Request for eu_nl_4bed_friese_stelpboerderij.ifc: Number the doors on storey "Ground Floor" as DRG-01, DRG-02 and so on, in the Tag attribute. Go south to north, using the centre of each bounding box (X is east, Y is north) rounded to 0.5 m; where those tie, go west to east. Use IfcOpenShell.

First a look at what the model holds.

```python
import ifcopenshell
import ifcopenshell.util.element
import ifcopenshell.util.placement

model = ifcopenshell.open("eu_nl_4bed_friese_stelpboerderij.ifc")
print(model.schema)
storey = next(s for s in model.by_type("IfcBuildingStorey") if s.Name == "Ground Floor")
doors = [e for e in ifcopenshell.util.element.get_decomposition(storey) if e.is_a("IfcDoor")]
for e in sorted(doors, key=lambda e: e.id()):
    origin = ifcopenshell.util.placement.get_local_placement(e.ObjectPlacement)[:3, 3]
    print(e.id(), e.Tag, e.Name, origin.round(2) + 0.0, sep=" | ")
```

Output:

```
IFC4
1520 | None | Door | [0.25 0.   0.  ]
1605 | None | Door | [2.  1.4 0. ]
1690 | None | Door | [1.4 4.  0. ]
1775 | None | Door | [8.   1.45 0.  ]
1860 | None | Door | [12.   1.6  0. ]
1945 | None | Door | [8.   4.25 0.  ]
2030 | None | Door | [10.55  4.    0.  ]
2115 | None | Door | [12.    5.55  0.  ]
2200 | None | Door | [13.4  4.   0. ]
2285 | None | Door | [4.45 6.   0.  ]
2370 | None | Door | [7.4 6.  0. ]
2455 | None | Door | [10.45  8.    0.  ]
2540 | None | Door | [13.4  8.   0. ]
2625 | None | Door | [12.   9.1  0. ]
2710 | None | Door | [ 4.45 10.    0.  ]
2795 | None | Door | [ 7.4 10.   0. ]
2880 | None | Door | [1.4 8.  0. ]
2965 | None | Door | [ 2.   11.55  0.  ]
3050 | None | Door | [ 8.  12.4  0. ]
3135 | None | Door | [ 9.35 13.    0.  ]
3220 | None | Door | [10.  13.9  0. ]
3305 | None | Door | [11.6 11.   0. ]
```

```python
import ifcopenshell
import ifcopenshell.geom
import ifcopenshell.util.element
import ifcopenshell.util.shape

model = ifcopenshell.open("eu_nl_4bed_friese_stelpboerderij.ifc")
settings = ifcopenshell.geom.settings()
settings.set("use-world-coords", True)


def centre(element):
    shape = ifcopenshell.geom.create_shape(settings, element)
    return ifcopenshell.util.shape.get_bbox_centroid(shape.geometry)


storey = next(s for s in model.by_type("IfcBuildingStorey") if s.Name == "Ground Floor")
doors = [e for e in ifcopenshell.util.element.get_decomposition(storey) if e.is_a("IfcDoor")]

# Insertion points can sit at a corner or the storey origin, so sort by the geometry (in metres).
centres = {e: centre(e) for e in doors}
doors.sort(key=lambda e: (round(centres[e][1] / 0.5), centres[e][0]))

for i, e in enumerate(doors, start=1):
    number = f"DRG-{i:02d}"
    e.Tag = number
    print(e.id(), number)

model.write("eu_nl_4bed_friese_stelpboerderij_rev.ifc")
```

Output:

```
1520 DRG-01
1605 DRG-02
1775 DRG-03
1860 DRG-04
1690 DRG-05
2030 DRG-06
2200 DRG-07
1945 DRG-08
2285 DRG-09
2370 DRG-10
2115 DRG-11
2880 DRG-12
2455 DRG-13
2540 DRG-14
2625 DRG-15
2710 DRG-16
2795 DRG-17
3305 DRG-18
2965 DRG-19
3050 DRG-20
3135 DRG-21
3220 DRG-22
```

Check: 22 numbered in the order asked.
